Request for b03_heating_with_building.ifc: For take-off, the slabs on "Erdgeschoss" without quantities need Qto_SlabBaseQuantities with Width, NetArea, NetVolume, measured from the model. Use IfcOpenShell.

First a look at what the model holds.

```python
import ifcopenshell
import ifcopenshell.util.element
import ifcopenshell.util.unit

model = ifcopenshell.open("b03_heating_with_building.ifc")
print(model.schema)
for unit_type in ("LENGTHUNIT", "AREAUNIT", "VOLUMEUNIT"):
    print(unit_type, ifcopenshell.util.unit.calculate_unit_scale(model, unit_type))
storey = next(s for s in model.by_type("IfcBuildingStorey") if s.Name == "Erdgeschoss")
slabs = [e for e in ifcopenshell.util.element.get_decomposition(storey) if e.is_a("IfcSlab")]
for e in sorted(slabs, key=lambda e: e.id()):
    print(e.id(), e.is_a(), e.Name, list(ifcopenshell.util.element.get_psets(e, qtos_only=True)), sep=" | ")
```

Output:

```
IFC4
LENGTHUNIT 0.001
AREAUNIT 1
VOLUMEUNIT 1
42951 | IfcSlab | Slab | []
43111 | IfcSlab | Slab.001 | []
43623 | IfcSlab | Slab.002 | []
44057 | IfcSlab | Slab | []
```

```python
import ifcopenshell
import ifcopenshell.api.pset
import ifcopenshell.geom
import ifcopenshell.util.element
import ifcopenshell.util.shape
import ifcopenshell.util.unit

model = ifcopenshell.open("b03_heating_with_building.ifc")
unit_scale = ifcopenshell.util.unit.calculate_unit_scale(model)
area_scale = ifcopenshell.util.unit.calculate_unit_scale(model, "AREAUNIT")
volume_scale = ifcopenshell.util.unit.calculate_unit_scale(model, "VOLUMEUNIT")
settings = ifcopenshell.geom.settings()

storey = next(s for s in model.by_type("IfcBuildingStorey") if s.Name == "Erdgeschoss")
slabs = [e for e in ifcopenshell.util.element.get_decomposition(storey) if e.is_a("IfcSlab")]

for e in sorted(slabs, key=lambda e: e.id()):
    if ifcopenshell.util.element.get_psets(e, qtos_only=True, should_inherit=False):
        continue
    # Geometry comes back in metres, in the element's own axes.
    shape = ifcopenshell.geom.create_shape(settings, e)
    values = {
        "Width": ifcopenshell.util.shape.get_z(shape.geometry) / unit_scale,
        "NetArea": ifcopenshell.util.shape.get_footprint_area(shape.geometry) / area_scale,
        "NetVolume": ifcopenshell.util.shape.get_volume(shape.geometry) / volume_scale,
    }
    qto = ifcopenshell.api.pset.add_qto(model, product=e, name="Qto_SlabBaseQuantities")
    ifcopenshell.api.pset.edit_qto(model, qto=qto, properties=values)
    print(e.id(), {k: round(v, 3) for k, v in values.items()})

model.write("b03_heating_with_building_edited.ifc")
```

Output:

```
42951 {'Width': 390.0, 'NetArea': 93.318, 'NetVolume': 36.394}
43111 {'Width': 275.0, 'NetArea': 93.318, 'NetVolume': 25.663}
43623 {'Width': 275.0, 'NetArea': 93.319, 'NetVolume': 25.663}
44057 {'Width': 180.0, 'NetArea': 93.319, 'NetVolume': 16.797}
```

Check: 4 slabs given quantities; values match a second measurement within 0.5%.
